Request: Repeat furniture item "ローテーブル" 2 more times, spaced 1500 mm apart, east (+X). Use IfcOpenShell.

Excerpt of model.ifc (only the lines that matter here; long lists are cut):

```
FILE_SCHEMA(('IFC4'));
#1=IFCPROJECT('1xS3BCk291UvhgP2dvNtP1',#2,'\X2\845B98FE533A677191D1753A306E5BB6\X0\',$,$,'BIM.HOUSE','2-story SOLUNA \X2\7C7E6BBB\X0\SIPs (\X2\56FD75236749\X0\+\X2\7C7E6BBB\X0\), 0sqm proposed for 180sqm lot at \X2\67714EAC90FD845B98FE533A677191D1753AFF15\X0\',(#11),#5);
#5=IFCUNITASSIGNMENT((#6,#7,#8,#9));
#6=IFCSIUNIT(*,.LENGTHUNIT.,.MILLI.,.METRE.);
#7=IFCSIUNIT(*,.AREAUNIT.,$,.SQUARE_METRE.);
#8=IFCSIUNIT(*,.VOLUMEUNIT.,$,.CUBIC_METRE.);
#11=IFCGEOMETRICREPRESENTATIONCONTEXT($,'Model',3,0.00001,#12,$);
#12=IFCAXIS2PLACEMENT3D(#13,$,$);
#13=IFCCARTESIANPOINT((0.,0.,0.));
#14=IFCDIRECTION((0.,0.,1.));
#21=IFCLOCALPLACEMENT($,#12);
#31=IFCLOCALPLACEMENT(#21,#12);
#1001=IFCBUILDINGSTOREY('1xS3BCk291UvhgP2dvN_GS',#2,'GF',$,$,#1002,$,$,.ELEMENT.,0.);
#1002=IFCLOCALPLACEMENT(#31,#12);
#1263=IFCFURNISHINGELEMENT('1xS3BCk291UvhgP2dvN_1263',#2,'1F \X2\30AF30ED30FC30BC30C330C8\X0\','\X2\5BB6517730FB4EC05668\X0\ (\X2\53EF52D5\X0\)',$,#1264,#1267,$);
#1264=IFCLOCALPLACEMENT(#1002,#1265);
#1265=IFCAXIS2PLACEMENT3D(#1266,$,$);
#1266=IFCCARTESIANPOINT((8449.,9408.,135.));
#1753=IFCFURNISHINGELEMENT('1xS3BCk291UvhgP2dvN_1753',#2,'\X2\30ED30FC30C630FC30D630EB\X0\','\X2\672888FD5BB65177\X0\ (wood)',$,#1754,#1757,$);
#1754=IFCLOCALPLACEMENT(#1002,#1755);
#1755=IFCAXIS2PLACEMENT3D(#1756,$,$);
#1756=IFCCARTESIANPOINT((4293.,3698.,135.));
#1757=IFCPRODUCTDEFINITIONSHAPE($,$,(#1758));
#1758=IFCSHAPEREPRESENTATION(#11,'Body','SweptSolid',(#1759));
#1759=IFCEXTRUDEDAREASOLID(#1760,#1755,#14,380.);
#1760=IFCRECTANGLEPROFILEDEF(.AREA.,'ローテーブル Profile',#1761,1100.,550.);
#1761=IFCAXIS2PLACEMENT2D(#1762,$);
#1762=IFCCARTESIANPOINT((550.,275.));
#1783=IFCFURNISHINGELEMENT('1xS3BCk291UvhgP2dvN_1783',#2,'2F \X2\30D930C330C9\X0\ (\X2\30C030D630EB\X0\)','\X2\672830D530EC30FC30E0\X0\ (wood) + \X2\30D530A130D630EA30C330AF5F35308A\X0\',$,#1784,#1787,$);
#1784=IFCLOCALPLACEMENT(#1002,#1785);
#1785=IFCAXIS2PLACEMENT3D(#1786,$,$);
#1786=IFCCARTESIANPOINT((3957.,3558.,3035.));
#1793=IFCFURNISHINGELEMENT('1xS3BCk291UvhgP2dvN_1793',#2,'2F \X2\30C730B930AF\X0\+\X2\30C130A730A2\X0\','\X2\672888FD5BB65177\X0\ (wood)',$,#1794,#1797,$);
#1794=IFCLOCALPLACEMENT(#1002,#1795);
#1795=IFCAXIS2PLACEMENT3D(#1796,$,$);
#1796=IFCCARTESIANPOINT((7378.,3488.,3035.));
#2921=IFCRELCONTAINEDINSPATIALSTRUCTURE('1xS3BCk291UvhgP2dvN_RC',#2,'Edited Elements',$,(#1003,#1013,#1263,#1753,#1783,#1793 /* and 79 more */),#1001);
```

```python
import numpy as np
import ifcopenshell
import ifcopenshell.api.geometry
import ifcopenshell.api.root
import ifcopenshell.util.element
import ifcopenshell.util.placement

model = ifcopenshell.open("model.ifc")


def reuse_history(source, copy):
    """copy_class also copies each property set's owner history, people and application; keep the originals."""
    for rel in copy.IsDefinedBy:
        if rel.is_a("IfcRelDefinesByProperties") and (history := rel.RelatingPropertyDefinition.OwnerHistory):
            rel.RelatingPropertyDefinition.OwnerHistory = source.OwnerHistory
            ifcopenshell.util.element.remove_deep2(model, history)


source = model.by_guid("1xS3BCk291UvhgP2dvN_1753")
base = ifcopenshell.util.placement.get_local_placement(source.ObjectPlacement)
step = np.array([1.0, 0.0, 0.0]) * 1500.0

for i in range(1, 3):
    copy = ifcopenshell.api.root.copy_class(model, product=source)
    copy.Representation = ifcopenshell.util.element.copy_deep(
        model, source.Representation, exclude=["IfcGeometricRepresentationContext", "IfcRepresentationMap"]
    )
    reuse_history(source, copy)
    matrix = base.copy()
    matrix[:3, 3] += i * step
    print("added at", matrix[:3, 3].round(3) + 0.0)
    ifcopenshell.api.geometry.edit_object_placement(model, product=copy, matrix=matrix, is_si=False)

model.write("model_v2.ifc")
```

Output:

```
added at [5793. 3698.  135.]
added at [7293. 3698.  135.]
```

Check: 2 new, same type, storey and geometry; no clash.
